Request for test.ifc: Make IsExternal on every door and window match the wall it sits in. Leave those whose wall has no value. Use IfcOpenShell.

First a look at what the model holds.

```python
import ifcopenshell
import ifcopenshell.util.element

model = ifcopenshell.open("test.ifc")
print(model.schema)
seen = {}
for e in model.by_type("IfcDoor") + model.by_type("IfcWindow"):
    if not e.FillsVoids:
        continue
    host = e.FillsVoids[0].RelatingOpeningElement.VoidsElements[0].RelatingBuildingElement
    own = ifcopenshell.util.element.get_pset(e, f"Pset_{e.is_a()[3:].removesuffix('StandardCase')}Common", "IsExternal")
    wall = ifcopenshell.util.element.get_pset(host, "Pset_WallCommon", "IsExternal")
    seen[e.is_a(), own, wall] = seen.get((e.is_a(), own, wall), 0) + 1
for (cls, own, wall), count in sorted(seen.items(), key=str):
    print(count, cls, "IsExternal:", own, "| host wall:", wall)
```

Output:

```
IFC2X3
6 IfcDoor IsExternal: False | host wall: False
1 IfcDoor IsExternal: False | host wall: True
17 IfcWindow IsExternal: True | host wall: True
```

```python
import ifcopenshell
import ifcopenshell.api.pset
import ifcopenshell.util.element

model = ifcopenshell.open("test.ifc")

count = 0
for ifc_class, pset_name in (("IfcDoor", "Pset_DoorCommon"), ("IfcWindow", "Pset_WindowCommon")):
    for e in model.by_type(ifc_class):
        if not e.FillsVoids:
            continue
        host = e.FillsVoids[0].RelatingOpeningElement.VoidsElements[0].RelatingBuildingElement
        external = ifcopenshell.util.element.get_pset(host, "Pset_WallCommon", "IsExternal")
        if external is None or ifcopenshell.util.element.get_pset(e, pset_name, "IsExternal") == external:
            continue
        pset = ifcopenshell.api.pset.add_pset(model, product=e, name=pset_name)
        ifcopenshell.api.pset.edit_pset(model, pset=pset, properties={"IsExternal": external})
        count += 1

print(count, "updated")

model.write("test-out.ifc")
```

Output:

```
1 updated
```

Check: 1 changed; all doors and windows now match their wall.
